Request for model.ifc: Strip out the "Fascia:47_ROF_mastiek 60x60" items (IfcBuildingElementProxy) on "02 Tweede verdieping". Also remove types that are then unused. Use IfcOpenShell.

First a look at what the model holds.

```python
import ifcopenshell
import ifcopenshell.util.element

model = ifcopenshell.open("model.ifc")
print(model.schema)
storey = next(s for s in model.by_type("IfcBuildingStorey") if s.Name == "02 Tweede verdieping")
proxies = [e for e in ifcopenshell.util.element.get_decomposition(storey) if e.is_a("IfcBuildingElementProxy")]
seen = {}
for e in proxies:
    element_type = ifcopenshell.util.element.get_type(e)
    name = element_type.Name if element_type not in (None, e) else None
    seen[name] = seen.get(name, 0) + 1
for name, count in sorted(seen.items(), key=str):
    print(count, "x", name)
```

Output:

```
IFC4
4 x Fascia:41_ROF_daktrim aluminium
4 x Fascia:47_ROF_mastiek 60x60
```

```python
import ifcopenshell
import ifcopenshell.api.root
import ifcopenshell.util.element

model = ifcopenshell.open("model.ifc")

storey = next(s for s in model.by_type("IfcBuildingStorey") if s.Name == "02 Tweede verdieping")
proxies = [e for e in ifcopenshell.util.element.get_decomposition(storey) if e.is_a("IfcBuildingElementProxy")]
targets = [e for e in proxies if (t := ifcopenshell.util.element.get_type(e)) not in (None, e) and t.Name == "Fascia:47_ROF_mastiek 60x60"]
types = {ifcopenshell.util.element.get_type(e) for e in targets} - {None, *targets}

for e in targets:
    ifcopenshell.api.root.remove_product(model, product=e)
print(len(targets), "removed")

unused = [t for t in types if not ifcopenshell.util.element.get_types(t)]
for t in unused:
    ifcopenshell.api.root.remove_product(model, product=t)
print(len(unused), "unused types removed")

model.write("model_v2.ifc")
```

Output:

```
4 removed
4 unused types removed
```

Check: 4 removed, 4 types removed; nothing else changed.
